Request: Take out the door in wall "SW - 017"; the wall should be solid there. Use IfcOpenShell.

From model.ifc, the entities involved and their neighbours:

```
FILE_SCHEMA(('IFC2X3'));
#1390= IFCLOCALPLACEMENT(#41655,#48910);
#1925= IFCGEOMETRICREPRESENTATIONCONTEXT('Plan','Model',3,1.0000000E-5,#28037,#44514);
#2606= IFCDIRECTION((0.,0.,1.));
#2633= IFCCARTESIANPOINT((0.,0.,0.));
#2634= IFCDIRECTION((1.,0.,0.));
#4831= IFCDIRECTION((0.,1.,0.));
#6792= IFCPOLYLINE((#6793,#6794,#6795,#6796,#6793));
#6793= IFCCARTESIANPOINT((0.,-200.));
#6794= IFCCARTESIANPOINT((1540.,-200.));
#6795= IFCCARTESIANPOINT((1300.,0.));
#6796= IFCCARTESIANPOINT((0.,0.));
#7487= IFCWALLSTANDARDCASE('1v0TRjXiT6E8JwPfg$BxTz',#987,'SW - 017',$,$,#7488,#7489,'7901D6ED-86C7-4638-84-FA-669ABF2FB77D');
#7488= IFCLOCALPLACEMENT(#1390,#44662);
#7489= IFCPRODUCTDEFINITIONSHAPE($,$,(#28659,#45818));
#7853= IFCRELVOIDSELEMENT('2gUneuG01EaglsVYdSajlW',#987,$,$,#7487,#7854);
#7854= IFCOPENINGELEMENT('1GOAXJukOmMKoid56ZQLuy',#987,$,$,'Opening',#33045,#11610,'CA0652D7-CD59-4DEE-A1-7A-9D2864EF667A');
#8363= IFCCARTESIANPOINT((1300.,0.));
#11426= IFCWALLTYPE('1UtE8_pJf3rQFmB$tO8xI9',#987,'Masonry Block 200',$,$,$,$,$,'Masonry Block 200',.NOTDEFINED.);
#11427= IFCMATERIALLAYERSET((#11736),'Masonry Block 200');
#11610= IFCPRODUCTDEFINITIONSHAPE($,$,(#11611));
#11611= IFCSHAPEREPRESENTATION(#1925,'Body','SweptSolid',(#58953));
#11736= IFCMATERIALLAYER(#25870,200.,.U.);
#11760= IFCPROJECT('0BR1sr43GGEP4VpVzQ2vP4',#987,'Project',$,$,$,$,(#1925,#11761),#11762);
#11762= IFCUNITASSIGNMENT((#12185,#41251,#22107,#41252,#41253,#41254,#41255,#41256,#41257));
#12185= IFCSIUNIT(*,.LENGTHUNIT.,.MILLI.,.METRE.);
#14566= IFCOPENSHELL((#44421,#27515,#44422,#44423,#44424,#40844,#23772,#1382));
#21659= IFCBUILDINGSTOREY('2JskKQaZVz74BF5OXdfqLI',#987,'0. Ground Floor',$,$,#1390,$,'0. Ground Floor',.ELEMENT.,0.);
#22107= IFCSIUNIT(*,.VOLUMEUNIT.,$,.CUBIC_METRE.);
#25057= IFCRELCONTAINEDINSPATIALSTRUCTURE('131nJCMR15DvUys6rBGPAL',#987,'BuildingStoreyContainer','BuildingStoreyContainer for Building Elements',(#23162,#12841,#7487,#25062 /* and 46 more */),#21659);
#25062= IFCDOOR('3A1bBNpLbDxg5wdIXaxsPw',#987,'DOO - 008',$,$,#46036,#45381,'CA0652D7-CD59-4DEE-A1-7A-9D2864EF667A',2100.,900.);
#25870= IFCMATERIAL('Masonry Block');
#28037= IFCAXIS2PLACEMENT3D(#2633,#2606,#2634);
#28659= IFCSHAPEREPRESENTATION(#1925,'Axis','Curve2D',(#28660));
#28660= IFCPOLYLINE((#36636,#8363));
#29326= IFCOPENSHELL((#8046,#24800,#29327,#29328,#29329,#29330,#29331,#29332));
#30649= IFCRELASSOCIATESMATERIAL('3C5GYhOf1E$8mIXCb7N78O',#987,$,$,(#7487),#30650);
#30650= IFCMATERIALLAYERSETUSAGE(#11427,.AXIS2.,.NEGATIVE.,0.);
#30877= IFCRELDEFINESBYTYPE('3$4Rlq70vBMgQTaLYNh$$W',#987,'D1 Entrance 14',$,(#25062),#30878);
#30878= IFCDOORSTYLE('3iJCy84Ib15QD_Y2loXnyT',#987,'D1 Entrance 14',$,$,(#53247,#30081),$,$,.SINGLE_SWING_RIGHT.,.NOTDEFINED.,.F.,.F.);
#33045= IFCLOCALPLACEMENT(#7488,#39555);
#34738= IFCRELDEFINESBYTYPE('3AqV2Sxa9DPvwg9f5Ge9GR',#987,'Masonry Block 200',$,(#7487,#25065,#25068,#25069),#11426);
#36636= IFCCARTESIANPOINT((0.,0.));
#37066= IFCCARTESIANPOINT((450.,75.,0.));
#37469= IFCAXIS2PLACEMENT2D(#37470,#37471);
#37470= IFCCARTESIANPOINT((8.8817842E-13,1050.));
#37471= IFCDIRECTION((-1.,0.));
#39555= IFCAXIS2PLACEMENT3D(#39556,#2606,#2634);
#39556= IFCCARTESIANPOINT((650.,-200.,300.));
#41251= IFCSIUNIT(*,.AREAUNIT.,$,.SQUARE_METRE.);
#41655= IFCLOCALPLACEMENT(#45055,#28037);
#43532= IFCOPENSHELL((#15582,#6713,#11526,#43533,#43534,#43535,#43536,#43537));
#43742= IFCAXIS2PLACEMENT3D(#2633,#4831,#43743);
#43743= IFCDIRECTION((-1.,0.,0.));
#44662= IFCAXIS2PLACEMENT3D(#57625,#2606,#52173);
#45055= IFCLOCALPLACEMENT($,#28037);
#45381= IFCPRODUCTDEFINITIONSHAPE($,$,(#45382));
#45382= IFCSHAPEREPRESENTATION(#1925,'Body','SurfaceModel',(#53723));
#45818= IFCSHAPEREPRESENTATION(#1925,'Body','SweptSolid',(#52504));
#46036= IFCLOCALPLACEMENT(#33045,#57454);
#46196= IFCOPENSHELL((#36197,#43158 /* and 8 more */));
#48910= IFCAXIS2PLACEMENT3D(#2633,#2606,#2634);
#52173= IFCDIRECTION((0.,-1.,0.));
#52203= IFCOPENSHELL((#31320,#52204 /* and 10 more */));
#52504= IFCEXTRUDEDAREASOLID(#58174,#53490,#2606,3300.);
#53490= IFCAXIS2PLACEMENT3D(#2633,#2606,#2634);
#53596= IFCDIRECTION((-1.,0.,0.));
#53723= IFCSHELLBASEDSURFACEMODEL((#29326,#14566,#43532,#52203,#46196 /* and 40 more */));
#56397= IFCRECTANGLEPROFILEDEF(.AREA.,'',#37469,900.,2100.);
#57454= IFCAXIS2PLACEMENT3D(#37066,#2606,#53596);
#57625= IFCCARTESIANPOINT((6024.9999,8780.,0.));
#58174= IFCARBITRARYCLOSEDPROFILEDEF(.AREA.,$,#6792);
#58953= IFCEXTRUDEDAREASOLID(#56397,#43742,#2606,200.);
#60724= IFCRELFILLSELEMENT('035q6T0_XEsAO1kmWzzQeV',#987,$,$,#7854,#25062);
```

```python
import ifcopenshell
import ifcopenshell.api.feature
import ifcopenshell.api.root
import ifcopenshell.geom
import ifcopenshell.util.shape

model = ifcopenshell.open("model.ifc")
settings = ifcopenshell.geom.settings()


def volume(element):
    """Net volume in cubic metres, openings subtracted."""
    shape = ifcopenshell.geom.create_shape(settings, element)
    return ifcopenshell.util.shape.get_volume(shape.geometry)


door = model.by_guid("3A1bBNpLbDxg5wdIXaxsPw")
opening = door.FillsVoids[0].RelatingOpeningElement
wall = opening.VoidsElements[0].RelatingBuildingElement
before = volume(wall)

ifcopenshell.api.root.remove_product(model, product=door)
ifcopenshell.api.feature.remove_feature(model, feature=opening)

after = volume(wall)

print(f"wall volume {before:.3f} -> {after:.3f} m3")

model.write("model-out.ifc")
```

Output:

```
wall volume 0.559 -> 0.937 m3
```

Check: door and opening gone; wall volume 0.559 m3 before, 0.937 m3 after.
